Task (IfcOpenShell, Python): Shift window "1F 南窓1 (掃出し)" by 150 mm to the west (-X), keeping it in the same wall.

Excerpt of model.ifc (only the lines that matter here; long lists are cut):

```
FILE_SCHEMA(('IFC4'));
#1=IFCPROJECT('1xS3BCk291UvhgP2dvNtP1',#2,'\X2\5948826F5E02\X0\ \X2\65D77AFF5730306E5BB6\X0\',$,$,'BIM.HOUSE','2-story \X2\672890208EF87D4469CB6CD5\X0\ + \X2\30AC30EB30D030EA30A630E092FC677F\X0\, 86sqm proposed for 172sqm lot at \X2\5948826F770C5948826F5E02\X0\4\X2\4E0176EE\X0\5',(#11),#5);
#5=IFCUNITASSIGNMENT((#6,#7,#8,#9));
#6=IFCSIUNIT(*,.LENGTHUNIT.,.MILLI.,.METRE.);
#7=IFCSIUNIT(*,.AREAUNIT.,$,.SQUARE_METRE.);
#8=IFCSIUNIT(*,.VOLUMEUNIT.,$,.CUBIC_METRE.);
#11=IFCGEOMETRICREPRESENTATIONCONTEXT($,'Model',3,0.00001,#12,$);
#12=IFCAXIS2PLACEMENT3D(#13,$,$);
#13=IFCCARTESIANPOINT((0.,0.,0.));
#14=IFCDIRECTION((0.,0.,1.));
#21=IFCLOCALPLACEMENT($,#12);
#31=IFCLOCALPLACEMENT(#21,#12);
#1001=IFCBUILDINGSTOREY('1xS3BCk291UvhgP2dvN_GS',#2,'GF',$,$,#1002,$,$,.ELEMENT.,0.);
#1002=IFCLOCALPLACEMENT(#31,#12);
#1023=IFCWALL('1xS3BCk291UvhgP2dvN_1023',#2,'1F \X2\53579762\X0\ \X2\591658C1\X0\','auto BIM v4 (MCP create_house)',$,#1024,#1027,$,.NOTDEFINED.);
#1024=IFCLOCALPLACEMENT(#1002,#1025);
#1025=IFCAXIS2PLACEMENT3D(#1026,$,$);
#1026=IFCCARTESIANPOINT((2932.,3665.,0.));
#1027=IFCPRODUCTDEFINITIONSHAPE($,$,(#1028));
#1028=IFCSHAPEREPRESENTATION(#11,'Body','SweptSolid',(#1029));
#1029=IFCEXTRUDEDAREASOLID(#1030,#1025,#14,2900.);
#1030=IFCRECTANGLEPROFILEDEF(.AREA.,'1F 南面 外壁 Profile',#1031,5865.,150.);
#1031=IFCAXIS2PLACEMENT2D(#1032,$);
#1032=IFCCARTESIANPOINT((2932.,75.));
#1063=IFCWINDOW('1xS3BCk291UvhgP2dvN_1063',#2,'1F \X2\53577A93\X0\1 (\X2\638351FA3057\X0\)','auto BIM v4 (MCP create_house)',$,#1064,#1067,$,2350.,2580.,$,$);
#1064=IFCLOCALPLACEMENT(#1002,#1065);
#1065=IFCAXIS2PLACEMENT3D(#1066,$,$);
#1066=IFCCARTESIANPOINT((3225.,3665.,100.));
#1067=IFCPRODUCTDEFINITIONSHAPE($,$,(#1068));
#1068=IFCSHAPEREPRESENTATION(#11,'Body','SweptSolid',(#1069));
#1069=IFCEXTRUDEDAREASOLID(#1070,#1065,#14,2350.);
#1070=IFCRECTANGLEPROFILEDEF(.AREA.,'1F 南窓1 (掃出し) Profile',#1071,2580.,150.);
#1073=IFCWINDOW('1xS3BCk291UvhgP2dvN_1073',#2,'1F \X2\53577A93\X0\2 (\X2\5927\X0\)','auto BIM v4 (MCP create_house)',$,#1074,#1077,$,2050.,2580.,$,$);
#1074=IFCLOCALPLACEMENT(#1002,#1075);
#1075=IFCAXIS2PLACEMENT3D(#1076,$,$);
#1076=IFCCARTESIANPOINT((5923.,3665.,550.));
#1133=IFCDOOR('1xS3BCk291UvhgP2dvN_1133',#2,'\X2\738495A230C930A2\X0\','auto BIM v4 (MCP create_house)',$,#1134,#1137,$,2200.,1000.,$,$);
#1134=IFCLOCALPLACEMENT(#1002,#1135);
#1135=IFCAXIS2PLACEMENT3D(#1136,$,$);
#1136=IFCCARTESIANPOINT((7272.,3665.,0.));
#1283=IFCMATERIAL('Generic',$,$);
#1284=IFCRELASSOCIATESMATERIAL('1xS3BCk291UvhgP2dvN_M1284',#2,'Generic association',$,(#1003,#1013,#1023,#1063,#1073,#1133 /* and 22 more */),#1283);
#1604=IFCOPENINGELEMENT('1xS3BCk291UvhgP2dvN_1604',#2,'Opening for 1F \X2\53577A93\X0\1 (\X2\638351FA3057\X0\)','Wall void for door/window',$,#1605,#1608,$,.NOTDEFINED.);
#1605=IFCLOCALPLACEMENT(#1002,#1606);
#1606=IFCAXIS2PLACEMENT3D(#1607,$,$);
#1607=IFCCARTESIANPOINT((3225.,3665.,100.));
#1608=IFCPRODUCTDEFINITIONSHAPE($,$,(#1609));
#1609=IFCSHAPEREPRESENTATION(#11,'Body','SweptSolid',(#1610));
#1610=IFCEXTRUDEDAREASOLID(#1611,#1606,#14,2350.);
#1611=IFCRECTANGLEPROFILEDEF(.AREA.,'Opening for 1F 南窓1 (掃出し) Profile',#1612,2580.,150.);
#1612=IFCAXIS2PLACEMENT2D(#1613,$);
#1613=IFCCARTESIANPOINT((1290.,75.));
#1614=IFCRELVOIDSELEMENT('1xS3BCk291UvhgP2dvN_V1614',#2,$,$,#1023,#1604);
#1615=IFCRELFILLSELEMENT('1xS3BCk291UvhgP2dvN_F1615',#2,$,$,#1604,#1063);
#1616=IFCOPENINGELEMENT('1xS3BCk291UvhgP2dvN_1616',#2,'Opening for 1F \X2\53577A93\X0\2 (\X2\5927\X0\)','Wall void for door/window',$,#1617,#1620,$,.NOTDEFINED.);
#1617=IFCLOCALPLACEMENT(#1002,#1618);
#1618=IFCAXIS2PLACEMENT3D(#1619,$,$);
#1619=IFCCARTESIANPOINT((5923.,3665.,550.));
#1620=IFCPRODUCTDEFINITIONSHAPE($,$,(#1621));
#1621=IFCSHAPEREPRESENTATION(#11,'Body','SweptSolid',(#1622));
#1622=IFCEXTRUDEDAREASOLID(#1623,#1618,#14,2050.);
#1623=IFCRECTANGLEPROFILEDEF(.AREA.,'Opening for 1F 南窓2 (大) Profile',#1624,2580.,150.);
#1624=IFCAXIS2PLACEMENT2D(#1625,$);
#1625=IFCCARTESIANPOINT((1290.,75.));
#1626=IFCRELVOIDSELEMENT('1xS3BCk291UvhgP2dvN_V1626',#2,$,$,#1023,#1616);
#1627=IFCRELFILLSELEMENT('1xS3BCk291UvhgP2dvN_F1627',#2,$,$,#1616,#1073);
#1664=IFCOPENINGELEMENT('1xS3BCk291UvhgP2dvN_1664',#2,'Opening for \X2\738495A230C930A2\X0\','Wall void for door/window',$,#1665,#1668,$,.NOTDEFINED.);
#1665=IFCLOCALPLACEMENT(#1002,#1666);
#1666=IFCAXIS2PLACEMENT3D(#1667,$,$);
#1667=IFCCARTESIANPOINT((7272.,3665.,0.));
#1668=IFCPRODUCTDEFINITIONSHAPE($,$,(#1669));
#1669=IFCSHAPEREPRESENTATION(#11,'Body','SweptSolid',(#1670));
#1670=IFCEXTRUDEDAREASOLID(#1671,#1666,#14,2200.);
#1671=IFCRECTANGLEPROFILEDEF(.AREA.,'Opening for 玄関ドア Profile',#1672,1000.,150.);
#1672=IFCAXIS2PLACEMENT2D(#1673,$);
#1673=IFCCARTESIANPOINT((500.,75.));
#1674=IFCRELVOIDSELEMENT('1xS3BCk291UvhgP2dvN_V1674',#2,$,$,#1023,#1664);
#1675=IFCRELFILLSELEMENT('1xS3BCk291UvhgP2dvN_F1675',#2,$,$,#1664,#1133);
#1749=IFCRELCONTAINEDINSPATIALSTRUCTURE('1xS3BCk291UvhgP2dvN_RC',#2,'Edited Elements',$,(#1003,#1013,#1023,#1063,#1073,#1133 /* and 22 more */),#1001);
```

```python
import ifcopenshell
import ifcopenshell.api.geometry
import ifcopenshell.util.placement

model = ifcopenshell.open("model.ifc")

window = model.by_guid("1xS3BCk291UvhgP2dvN_1063")
opening = window.FillsVoids[0].RelatingOpeningElement
wall = opening.VoidsElements[0].RelatingBuildingElement

wall_matrix = ifcopenshell.util.placement.get_local_placement(wall.ObjectPlacement)
shift = wall_matrix[:3, 0] * -150.0
before = ifcopenshell.util.placement.get_local_placement(window.ObjectPlacement)[:3, 3].copy()

# The window is not placed relative to its opening, so move both.
for product in (opening, window):
    matrix = ifcopenshell.util.placement.get_local_placement(product.ObjectPlacement)
    matrix[:3, 3] += shift
    ifcopenshell.api.geometry.edit_object_placement(model, product=product, matrix=matrix, is_si=False)

after = ifcopenshell.util.placement.get_local_placement(window.ObjectPlacement)[:3, 3]
print("window moved by", (after - before).round(3) + 0.0)

model.write("model-out.ifc")
```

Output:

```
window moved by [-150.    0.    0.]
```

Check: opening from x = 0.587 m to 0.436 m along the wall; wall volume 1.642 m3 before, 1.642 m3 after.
